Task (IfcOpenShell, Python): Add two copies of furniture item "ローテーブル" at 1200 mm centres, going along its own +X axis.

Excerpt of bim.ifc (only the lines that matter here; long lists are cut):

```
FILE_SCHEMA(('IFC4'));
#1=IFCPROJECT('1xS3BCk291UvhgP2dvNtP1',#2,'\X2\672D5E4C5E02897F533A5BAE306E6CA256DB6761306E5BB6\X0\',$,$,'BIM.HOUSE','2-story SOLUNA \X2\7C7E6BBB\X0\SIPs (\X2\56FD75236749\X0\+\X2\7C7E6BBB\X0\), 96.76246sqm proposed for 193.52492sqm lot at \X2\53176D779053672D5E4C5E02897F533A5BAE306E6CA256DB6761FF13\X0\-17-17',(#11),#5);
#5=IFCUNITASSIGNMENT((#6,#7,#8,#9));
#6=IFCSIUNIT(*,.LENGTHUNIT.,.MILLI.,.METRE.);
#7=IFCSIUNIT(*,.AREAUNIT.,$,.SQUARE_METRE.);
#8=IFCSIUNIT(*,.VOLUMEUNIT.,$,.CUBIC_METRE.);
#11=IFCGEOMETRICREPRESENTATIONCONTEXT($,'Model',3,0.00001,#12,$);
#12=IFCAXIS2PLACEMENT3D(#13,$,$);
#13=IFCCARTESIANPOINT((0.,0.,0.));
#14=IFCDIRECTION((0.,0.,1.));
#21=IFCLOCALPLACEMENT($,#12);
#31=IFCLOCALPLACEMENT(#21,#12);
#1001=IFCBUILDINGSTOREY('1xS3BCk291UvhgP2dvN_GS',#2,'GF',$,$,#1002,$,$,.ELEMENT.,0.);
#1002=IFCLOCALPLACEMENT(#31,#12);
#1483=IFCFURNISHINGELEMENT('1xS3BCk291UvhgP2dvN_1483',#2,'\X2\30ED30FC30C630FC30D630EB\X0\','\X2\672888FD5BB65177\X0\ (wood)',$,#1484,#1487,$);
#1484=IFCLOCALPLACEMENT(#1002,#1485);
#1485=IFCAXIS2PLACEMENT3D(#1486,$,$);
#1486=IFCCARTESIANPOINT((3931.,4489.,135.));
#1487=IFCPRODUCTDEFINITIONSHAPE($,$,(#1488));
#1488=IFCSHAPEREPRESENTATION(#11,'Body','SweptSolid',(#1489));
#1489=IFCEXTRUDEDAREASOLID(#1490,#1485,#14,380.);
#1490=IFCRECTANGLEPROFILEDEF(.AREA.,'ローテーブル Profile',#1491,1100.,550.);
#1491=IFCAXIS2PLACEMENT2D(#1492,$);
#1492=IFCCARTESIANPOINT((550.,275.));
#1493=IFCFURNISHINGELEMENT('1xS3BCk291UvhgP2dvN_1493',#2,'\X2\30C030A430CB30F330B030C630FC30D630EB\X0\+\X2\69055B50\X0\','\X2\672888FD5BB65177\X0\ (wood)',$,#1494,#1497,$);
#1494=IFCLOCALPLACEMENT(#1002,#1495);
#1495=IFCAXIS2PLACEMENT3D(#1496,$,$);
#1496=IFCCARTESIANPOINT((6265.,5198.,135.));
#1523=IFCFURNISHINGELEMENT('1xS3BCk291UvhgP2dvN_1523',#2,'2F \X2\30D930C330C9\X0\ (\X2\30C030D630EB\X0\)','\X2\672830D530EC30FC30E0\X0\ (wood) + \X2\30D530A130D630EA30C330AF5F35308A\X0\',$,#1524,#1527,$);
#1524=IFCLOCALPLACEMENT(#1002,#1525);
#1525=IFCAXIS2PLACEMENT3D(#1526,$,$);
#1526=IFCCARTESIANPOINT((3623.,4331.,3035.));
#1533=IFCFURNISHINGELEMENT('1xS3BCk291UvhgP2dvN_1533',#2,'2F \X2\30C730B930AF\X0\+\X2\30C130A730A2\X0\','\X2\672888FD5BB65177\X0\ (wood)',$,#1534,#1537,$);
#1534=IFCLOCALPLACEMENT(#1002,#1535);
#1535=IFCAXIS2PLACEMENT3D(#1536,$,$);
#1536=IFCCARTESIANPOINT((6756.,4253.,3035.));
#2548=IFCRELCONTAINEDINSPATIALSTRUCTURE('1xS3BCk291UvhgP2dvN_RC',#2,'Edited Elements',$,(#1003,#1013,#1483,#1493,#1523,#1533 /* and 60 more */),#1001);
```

```python
import ifcopenshell
import ifcopenshell.api.geometry
import ifcopenshell.api.root
import ifcopenshell.util.element
import ifcopenshell.util.placement

model = ifcopenshell.open("bim.ifc")


def reuse_history(source, copy):
    """copy_class also copies each property set's owner history, people and application; keep the originals."""
    for rel in copy.IsDefinedBy:
        if rel.is_a("IfcRelDefinesByProperties") and (history := rel.RelatingPropertyDefinition.OwnerHistory):
            rel.RelatingPropertyDefinition.OwnerHistory = source.OwnerHistory
            ifcopenshell.util.element.remove_deep2(model, history)


source = model.by_guid("1xS3BCk291UvhgP2dvN_1483")
base = ifcopenshell.util.placement.get_local_placement(source.ObjectPlacement)
step = base[:3, 0] * 1200.0

for i in range(1, 3):
    copy = ifcopenshell.api.root.copy_class(model, product=source)
    copy.Representation = ifcopenshell.util.element.copy_deep(
        model, source.Representation, exclude=["IfcGeometricRepresentationContext", "IfcRepresentationMap"]
    )
    reuse_history(source, copy)
    matrix = base.copy()
    matrix[:3, 3] += i * step
    print("added at", matrix[:3, 3].round(3) + 0.0)
    ifcopenshell.api.geometry.edit_object_placement(model, product=copy, matrix=matrix, is_si=False)

model.write("bim_updated.ifc")
```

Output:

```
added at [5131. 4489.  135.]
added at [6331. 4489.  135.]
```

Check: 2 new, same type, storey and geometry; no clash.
